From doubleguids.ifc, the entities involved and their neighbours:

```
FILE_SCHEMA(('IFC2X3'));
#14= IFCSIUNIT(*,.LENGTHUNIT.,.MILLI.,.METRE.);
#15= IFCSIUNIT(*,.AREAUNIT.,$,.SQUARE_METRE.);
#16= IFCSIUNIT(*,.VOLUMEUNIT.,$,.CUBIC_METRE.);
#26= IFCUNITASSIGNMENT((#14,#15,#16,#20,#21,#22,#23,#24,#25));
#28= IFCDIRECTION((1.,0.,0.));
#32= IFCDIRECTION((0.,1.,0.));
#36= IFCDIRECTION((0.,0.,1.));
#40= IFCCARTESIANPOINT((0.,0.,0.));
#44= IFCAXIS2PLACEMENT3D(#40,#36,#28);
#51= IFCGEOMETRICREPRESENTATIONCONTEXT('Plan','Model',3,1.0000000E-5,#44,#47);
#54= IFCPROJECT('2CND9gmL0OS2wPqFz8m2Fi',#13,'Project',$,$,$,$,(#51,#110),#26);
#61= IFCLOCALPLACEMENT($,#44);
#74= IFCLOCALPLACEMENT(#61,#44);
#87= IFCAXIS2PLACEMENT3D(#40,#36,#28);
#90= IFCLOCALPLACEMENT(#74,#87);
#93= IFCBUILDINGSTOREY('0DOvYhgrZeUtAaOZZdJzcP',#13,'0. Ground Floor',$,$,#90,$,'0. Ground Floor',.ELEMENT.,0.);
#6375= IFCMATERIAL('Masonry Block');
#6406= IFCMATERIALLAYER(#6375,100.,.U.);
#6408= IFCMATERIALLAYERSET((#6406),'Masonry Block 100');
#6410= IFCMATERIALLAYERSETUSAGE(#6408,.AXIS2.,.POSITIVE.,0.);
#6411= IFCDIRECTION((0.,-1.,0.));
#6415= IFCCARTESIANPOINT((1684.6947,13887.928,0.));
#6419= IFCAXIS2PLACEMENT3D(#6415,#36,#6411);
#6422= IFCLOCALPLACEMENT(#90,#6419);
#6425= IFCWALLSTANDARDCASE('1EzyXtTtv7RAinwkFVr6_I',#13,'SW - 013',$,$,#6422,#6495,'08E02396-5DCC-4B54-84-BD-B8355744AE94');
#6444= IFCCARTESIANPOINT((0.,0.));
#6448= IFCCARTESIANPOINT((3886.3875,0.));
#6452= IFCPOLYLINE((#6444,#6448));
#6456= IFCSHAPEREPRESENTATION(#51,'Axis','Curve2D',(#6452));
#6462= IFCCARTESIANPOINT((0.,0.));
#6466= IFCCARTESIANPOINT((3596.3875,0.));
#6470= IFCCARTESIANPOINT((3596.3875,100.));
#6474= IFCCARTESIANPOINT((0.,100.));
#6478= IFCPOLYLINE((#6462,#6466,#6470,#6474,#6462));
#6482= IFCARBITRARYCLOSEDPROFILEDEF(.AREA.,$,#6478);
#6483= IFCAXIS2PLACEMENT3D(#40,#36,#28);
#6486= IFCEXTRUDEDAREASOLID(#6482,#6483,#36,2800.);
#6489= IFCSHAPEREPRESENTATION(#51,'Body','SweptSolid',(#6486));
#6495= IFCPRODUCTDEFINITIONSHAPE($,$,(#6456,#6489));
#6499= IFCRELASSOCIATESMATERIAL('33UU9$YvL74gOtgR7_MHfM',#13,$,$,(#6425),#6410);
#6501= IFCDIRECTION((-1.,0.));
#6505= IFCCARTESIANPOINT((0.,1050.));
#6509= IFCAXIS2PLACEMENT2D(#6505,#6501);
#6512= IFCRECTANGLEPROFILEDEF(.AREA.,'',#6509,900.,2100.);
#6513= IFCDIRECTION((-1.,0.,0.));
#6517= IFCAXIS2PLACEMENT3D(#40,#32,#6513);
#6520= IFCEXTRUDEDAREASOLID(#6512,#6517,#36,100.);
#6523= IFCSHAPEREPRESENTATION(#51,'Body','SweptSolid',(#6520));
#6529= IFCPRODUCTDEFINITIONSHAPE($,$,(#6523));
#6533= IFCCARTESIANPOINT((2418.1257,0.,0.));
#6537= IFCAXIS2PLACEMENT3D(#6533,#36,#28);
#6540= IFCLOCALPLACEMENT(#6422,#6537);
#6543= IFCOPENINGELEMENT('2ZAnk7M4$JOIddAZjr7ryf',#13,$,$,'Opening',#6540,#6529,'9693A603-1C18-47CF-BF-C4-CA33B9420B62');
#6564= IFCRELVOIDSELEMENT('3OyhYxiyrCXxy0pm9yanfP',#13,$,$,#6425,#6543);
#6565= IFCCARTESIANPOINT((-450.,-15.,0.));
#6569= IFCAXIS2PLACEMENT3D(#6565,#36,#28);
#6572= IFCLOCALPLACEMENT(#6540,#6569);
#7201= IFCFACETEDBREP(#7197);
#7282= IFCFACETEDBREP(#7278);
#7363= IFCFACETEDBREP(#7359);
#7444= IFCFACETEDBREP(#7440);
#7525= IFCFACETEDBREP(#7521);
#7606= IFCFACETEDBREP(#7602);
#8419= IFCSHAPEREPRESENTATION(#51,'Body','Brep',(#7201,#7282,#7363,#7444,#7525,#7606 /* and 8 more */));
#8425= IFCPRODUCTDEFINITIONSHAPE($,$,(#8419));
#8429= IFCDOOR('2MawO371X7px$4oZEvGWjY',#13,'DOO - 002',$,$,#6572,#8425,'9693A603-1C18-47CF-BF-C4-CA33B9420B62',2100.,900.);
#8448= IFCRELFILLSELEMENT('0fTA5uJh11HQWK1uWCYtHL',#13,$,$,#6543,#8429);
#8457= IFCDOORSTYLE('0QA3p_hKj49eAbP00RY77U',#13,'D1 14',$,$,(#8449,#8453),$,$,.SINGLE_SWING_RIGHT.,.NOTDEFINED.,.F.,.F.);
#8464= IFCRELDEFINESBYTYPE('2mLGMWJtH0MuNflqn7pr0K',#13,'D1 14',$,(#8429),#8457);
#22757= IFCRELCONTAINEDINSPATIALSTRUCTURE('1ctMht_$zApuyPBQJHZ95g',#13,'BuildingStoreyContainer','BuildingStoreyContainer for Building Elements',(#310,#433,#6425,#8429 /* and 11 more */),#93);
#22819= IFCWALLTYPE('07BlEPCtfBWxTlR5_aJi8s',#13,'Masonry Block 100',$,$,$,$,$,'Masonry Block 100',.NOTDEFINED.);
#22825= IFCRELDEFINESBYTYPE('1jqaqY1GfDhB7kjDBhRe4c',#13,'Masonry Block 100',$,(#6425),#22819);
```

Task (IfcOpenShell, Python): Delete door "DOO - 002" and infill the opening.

```python
import ifcopenshell
import ifcopenshell.api.feature
import ifcopenshell.api.root
import ifcopenshell.geom
import ifcopenshell.util.shape

model = ifcopenshell.open("doubleguids.ifc")
settings = ifcopenshell.geom.settings()


def volume(element):
    """Net volume in cubic metres, openings subtracted."""
    shape = ifcopenshell.geom.create_shape(settings, element)
    return ifcopenshell.util.shape.get_volume(shape.geometry)


door = model.by_id(8429)
opening = door.FillsVoids[0].RelatingOpeningElement
wall = opening.VoidsElements[0].RelatingBuildingElement
before = volume(wall)

ifcopenshell.api.root.remove_product(model, product=door)
ifcopenshell.api.feature.remove_feature(model, feature=opening)

after = volume(wall)

print(f"wall volume {before:.3f} -> {after:.3f} m3")

model.write("doubleguids_edited.ifc")
```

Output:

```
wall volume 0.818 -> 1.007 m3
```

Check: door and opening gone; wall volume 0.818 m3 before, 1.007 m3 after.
